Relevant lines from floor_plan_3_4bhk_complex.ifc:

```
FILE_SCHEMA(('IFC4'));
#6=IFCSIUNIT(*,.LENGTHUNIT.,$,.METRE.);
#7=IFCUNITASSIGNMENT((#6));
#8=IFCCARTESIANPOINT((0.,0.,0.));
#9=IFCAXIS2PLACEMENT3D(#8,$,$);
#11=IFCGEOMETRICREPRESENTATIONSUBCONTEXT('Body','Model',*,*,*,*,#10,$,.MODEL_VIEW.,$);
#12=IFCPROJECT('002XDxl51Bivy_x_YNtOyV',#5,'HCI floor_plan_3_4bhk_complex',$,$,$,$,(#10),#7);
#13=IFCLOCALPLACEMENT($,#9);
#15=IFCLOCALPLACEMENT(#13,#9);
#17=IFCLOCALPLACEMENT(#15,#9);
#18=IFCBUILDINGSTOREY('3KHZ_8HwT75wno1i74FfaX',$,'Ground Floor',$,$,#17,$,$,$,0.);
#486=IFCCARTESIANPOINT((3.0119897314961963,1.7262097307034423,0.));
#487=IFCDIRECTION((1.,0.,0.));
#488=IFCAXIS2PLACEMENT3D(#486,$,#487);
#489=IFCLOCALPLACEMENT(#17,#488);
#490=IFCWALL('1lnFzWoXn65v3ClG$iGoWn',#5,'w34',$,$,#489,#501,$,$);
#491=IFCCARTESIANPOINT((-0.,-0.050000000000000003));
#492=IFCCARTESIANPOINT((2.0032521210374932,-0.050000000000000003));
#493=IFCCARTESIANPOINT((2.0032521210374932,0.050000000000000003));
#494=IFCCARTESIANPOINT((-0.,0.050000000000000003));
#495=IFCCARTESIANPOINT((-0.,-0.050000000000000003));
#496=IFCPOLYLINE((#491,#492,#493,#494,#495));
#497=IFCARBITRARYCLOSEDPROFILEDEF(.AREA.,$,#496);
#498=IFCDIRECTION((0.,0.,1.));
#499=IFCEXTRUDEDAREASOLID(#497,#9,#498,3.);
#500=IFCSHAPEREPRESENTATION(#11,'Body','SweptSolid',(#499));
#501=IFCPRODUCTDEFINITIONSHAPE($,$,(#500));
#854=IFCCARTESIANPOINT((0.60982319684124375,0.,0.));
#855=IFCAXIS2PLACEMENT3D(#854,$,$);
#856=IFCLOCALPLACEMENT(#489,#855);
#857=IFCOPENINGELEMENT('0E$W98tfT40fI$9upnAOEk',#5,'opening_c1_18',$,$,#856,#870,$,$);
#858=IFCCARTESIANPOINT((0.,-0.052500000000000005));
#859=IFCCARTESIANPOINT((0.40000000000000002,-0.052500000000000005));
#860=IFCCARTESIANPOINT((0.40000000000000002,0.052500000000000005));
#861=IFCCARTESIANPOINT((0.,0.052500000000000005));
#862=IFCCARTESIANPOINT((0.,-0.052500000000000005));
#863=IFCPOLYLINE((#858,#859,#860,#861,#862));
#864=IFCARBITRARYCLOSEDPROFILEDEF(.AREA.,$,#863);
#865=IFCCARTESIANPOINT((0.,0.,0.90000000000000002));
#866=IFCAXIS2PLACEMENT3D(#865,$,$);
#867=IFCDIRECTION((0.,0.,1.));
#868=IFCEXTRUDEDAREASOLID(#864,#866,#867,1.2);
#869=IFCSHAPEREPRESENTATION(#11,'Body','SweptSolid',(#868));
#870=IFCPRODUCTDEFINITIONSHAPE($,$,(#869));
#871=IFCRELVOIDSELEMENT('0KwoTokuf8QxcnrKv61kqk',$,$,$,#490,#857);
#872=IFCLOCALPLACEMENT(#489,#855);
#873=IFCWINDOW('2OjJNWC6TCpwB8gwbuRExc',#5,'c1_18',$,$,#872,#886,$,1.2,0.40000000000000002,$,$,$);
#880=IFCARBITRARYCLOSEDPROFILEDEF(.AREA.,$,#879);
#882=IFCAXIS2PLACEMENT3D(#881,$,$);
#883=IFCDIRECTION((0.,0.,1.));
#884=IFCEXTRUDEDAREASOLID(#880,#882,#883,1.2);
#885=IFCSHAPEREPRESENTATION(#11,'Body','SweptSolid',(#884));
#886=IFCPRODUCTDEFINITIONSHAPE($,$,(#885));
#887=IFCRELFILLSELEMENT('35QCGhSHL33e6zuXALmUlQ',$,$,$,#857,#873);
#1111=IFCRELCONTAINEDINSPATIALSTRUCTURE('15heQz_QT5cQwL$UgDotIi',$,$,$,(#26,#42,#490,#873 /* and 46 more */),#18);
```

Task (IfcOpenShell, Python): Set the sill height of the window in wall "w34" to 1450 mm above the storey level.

```python
import numpy as np
import ifcopenshell
import ifcopenshell.api.geometry
import ifcopenshell.geom
import ifcopenshell.util.element
import ifcopenshell.util.placement
import ifcopenshell.util.shape
import ifcopenshell.util.unit

model = ifcopenshell.open("floor_plan_3_4bhk_complex.ifc")
unit_scale = ifcopenshell.util.unit.calculate_unit_scale(model)

window = model.by_guid("2OjJNWC6TCpwB8gwbuRExc")
opening = window.FillsVoids[0].RelatingOpeningElement
storey = ifcopenshell.util.element.get_container(window, ifc_class="IfcBuildingStorey")
level = ifcopenshell.util.placement.get_local_placement(storey.ObjectPlacement)[2, 3]

# The opening's origin need not be at the sill, so measure its lowest point.
shape = ifcopenshell.geom.create_shape(ifcopenshell.geom.settings(), opening)
bottom = ifcopenshell.util.shape.get_shape_bottom_elevation(shape, shape.geometry) / unit_scale
dz = level + 1.45 / unit_scale - bottom

shift = np.array([0.0, 0.0, dz])
# The window is not placed relative to its opening, so move both.
for product in (opening, window):
    matrix = ifcopenshell.util.placement.get_local_placement(product.ObjectPlacement)
    matrix[:3, 3] += shift
    ifcopenshell.api.geometry.edit_object_placement(model, product=product, matrix=matrix, is_si=False)

print(f"moved by {dz * unit_scale:+.3f} m")

model.write("floor_plan_3_4bhk_complex_v2.ifc")
```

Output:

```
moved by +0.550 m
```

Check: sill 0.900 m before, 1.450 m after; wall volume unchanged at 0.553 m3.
